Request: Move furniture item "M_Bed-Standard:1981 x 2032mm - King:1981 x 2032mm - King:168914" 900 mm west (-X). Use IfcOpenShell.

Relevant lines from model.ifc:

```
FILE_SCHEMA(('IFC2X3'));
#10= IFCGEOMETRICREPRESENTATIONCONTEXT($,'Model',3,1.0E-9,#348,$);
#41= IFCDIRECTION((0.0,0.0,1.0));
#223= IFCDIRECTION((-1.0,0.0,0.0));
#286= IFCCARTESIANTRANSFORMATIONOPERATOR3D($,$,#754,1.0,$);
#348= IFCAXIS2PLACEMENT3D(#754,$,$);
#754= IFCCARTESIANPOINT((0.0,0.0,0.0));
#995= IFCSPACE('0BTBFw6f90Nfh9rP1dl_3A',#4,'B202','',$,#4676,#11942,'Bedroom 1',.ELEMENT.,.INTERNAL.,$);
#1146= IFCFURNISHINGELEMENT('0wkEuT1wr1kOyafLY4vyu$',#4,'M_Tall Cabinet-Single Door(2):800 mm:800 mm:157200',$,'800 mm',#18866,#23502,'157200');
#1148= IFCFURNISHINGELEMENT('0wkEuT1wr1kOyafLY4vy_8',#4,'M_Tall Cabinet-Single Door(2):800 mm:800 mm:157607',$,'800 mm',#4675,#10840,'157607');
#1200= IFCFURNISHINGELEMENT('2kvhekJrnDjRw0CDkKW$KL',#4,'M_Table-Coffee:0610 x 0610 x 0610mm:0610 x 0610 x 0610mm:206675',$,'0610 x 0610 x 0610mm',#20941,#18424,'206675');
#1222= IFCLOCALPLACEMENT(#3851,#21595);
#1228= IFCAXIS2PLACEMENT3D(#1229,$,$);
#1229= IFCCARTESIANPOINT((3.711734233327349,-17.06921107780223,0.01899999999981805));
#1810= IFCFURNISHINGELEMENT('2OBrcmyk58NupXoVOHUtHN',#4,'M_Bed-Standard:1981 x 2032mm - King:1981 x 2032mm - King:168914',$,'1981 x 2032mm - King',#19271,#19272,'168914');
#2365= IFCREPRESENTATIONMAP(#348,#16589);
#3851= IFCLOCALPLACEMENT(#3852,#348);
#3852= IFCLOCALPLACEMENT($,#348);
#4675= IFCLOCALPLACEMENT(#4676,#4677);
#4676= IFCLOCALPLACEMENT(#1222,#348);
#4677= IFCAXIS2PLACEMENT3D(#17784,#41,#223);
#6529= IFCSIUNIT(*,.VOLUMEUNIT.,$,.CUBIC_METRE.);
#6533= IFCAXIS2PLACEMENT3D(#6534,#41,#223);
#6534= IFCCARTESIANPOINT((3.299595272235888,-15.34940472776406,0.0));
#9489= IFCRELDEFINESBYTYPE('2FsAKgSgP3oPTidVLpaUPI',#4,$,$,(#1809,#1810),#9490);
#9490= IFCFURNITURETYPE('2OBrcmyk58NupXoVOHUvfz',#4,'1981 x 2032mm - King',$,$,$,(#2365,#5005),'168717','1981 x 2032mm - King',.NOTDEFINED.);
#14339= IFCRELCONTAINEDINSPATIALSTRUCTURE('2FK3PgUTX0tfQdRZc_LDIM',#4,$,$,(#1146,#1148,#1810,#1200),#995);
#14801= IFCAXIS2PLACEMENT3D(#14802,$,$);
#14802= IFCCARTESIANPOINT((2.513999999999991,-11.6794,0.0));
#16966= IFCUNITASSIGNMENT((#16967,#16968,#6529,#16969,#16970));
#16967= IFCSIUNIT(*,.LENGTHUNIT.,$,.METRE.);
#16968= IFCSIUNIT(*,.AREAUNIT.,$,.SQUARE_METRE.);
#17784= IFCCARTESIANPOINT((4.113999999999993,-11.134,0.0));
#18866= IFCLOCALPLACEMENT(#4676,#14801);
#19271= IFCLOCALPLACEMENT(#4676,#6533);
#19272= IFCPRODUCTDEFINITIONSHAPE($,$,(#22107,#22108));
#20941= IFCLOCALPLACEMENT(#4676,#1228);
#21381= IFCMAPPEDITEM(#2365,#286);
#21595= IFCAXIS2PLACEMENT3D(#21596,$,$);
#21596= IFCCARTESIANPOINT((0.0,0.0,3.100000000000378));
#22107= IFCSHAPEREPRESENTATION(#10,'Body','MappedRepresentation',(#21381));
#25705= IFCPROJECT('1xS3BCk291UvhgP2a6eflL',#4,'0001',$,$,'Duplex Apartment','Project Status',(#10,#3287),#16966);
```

```python
import ifcopenshell
import ifcopenshell.api.geometry
import ifcopenshell.util.placement

model = ifcopenshell.open("model.ifc")

item = model.by_guid("2OBrcmyk58NupXoVOHUtHN")
matrix = ifcopenshell.util.placement.get_local_placement(item.ObjectPlacement)
matrix[0, 3] -= 0.9
ifcopenshell.api.geometry.edit_object_placement(model, product=item, matrix=matrix, is_si=False)

print(ifcopenshell.util.placement.get_local_placement(item.ObjectPlacement).round(3) + 0.0)

model.write("model_rev.ifc")
```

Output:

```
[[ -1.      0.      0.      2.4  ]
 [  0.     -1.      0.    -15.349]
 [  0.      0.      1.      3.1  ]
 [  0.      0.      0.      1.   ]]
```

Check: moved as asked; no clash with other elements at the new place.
